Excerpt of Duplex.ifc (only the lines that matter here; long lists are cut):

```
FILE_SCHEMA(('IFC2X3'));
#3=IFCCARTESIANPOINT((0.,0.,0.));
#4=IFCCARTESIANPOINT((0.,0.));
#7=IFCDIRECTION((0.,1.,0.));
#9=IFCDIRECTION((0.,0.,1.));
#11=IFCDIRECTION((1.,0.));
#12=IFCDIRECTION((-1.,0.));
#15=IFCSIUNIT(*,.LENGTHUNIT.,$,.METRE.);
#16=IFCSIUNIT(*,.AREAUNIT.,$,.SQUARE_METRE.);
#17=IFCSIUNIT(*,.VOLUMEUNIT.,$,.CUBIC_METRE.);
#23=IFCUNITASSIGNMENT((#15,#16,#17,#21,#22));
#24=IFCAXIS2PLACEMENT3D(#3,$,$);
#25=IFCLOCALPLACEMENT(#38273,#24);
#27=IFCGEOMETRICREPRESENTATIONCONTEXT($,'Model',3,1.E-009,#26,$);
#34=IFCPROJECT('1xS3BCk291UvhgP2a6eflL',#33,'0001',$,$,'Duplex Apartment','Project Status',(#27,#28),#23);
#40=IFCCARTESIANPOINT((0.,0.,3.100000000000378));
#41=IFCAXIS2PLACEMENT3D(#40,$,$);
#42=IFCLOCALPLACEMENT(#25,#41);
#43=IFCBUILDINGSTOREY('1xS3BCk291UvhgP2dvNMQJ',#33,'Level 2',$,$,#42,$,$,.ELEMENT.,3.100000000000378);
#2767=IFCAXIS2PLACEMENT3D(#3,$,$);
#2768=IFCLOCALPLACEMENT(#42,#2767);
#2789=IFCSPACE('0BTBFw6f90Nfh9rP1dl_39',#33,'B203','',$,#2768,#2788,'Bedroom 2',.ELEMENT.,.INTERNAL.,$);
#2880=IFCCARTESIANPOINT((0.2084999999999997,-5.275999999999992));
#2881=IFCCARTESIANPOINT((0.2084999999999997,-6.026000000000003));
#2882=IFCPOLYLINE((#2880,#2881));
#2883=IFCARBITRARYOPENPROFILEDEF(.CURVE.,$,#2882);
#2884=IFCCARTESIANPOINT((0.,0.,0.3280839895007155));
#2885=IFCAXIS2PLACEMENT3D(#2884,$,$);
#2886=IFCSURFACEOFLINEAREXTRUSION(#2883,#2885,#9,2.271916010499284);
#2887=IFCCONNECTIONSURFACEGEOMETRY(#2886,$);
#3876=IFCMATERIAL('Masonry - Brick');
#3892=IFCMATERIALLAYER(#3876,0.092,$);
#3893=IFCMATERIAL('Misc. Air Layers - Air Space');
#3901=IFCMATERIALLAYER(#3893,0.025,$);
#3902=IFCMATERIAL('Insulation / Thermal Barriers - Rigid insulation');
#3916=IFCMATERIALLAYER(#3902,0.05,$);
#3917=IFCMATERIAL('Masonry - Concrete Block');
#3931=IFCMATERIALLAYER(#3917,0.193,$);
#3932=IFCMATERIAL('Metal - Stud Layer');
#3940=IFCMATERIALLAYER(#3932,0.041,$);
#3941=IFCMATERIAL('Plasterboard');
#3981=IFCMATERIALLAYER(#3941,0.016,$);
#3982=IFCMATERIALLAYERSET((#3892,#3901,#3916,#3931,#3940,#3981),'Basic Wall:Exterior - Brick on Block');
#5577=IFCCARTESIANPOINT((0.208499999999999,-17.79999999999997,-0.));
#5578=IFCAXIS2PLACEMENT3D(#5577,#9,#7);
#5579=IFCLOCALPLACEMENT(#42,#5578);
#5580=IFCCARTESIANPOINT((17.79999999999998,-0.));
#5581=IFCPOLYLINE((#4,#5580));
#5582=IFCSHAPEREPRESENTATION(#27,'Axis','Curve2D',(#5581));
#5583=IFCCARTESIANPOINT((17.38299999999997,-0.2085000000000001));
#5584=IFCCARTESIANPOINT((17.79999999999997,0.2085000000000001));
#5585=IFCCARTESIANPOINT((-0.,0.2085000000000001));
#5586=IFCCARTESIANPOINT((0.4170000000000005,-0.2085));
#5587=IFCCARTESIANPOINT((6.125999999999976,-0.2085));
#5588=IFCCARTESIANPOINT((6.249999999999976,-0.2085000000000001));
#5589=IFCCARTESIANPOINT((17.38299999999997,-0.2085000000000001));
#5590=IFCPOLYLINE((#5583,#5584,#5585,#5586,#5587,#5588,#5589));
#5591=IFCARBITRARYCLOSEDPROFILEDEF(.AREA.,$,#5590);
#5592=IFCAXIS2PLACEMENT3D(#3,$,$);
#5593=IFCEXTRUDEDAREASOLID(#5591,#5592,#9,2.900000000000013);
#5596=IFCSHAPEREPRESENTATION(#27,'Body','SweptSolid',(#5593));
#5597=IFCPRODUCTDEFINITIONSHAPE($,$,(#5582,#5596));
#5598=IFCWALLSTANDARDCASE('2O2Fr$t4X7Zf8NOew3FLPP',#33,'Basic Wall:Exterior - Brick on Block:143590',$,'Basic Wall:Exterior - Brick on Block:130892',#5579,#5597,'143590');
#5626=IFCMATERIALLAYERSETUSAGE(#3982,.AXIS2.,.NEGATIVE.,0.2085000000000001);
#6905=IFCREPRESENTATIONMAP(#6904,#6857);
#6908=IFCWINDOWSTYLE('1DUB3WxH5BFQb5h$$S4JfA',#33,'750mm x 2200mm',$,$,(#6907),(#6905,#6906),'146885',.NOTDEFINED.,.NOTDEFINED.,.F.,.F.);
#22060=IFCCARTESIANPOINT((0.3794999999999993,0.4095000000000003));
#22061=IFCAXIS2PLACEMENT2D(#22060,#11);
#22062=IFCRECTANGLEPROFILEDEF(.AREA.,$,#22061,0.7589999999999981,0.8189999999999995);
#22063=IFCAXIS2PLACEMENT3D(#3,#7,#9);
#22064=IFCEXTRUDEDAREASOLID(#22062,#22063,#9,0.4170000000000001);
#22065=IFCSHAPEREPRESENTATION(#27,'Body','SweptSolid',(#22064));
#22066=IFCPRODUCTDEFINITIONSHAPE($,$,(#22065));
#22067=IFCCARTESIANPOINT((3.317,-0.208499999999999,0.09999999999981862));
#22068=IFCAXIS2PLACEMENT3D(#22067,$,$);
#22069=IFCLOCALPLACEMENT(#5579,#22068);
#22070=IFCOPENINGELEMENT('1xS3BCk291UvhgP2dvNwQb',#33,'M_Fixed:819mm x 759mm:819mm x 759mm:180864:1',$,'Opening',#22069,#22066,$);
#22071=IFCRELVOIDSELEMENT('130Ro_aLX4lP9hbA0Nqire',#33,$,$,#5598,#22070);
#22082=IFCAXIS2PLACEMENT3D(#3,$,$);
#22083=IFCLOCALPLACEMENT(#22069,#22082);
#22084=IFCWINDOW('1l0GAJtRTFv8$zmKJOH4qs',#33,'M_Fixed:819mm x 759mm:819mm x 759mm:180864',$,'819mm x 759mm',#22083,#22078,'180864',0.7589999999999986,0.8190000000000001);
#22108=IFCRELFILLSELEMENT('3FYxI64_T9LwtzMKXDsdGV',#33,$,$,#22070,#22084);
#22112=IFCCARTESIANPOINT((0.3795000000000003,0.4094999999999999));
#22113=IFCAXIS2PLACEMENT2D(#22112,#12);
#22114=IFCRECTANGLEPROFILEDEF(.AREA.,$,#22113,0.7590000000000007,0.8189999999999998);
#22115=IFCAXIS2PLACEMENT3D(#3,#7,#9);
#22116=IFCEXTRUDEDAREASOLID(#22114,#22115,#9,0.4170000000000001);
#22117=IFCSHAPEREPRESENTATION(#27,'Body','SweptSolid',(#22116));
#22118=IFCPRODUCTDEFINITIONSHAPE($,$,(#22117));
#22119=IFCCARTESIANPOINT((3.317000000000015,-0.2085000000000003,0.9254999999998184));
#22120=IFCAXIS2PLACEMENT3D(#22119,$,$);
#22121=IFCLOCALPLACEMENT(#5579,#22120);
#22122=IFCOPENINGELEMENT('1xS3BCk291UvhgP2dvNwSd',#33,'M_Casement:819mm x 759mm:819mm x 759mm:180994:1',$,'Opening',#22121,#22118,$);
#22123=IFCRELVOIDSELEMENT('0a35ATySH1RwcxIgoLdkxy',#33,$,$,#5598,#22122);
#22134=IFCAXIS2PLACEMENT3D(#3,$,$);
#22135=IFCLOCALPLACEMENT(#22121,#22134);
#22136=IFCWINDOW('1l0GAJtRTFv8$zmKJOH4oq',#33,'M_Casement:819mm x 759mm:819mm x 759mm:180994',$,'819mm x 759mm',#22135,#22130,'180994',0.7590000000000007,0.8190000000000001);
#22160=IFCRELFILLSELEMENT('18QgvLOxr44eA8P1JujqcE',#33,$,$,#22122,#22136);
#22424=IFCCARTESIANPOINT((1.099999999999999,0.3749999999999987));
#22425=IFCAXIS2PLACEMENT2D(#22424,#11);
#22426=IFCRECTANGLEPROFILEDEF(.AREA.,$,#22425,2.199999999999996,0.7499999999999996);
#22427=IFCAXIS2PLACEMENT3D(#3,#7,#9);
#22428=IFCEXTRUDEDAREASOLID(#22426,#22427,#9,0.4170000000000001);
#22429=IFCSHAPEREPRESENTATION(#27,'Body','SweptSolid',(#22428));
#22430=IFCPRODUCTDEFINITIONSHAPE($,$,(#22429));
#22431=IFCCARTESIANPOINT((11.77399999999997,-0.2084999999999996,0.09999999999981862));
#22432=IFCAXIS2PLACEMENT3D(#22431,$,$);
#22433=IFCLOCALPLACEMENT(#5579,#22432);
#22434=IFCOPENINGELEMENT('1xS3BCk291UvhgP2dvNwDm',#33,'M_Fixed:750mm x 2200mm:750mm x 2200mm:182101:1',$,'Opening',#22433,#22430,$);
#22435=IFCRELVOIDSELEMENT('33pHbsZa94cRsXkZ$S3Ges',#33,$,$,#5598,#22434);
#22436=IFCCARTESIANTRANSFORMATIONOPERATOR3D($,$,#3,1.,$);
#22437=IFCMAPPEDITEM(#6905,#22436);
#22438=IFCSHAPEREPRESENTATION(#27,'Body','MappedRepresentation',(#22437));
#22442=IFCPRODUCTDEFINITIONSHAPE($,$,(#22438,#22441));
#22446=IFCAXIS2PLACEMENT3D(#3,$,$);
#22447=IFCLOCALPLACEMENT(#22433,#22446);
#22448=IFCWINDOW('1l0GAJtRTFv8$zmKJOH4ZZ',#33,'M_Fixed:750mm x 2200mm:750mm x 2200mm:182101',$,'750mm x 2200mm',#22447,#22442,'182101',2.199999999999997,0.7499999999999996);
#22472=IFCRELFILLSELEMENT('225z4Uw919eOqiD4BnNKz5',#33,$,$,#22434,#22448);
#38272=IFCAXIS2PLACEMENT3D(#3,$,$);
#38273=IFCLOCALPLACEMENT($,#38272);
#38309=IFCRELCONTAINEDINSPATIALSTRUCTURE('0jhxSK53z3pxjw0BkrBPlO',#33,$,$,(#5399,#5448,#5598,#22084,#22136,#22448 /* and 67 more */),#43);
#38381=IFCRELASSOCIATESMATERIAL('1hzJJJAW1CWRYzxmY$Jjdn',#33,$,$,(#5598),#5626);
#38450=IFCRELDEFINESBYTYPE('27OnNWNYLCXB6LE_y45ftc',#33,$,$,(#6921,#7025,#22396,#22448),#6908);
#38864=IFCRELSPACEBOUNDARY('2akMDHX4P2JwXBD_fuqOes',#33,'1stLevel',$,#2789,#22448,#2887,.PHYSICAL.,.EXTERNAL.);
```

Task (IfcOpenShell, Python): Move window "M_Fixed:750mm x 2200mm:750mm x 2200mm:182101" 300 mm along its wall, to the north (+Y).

```python
import numpy as np
import ifcopenshell
import ifcopenshell.api.geometry
import ifcopenshell.util.placement
import ifcopenshell.util.unit

model = ifcopenshell.open("Duplex.ifc")
unit_scale = ifcopenshell.util.unit.calculate_unit_scale(model)

window = model.by_id(22448)
opening = window.FillsVoids[0].RelatingOpeningElement
wall = opening.VoidsElements[0].RelatingBuildingElement

wall_matrix = ifcopenshell.util.placement.get_local_placement(wall.ObjectPlacement)
shift = wall_matrix[:3, 0] * 0.3 / unit_scale
before = ifcopenshell.util.placement.get_local_placement(window.ObjectPlacement)[:3, 3].copy()

# The window is placed relative to its opening, so it follows when the opening moves.
matrix = ifcopenshell.util.placement.get_local_placement(opening.ObjectPlacement)
matrix[:3, 3] += shift
ifcopenshell.api.geometry.edit_object_placement(
    model, product=opening, matrix=matrix, is_si=False, should_transform_children=True
)

# Space boundary surfaces are stored in each space's coordinates; move them too.
for rel in window.ProvidesBoundaries:
    if not rel.ConnectionGeometry:
        continue
    surface = rel.ConnectionGeometry.SurfaceOnRelatingElement
    space_matrix = ifcopenshell.util.placement.get_local_placement(rel.RelatingSpace.ObjectPlacement)
    point = np.array(surface.Position.Location.Coordinates) + space_matrix[:3, :3].T @ shift
    surface.Position = model.createIfcAxis2Placement3D(
        model.createIfcCartesianPoint(point.tolist()), surface.Position.Axis, surface.Position.RefDirection
    )

after = ifcopenshell.util.placement.get_local_placement(window.ObjectPlacement)[:3, 3]
print("window moved by", (after - before).round(3) + 0.0)

model.write("Duplex_updated.ifc")
```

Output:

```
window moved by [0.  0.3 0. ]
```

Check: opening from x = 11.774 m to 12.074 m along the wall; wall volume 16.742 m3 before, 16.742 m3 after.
